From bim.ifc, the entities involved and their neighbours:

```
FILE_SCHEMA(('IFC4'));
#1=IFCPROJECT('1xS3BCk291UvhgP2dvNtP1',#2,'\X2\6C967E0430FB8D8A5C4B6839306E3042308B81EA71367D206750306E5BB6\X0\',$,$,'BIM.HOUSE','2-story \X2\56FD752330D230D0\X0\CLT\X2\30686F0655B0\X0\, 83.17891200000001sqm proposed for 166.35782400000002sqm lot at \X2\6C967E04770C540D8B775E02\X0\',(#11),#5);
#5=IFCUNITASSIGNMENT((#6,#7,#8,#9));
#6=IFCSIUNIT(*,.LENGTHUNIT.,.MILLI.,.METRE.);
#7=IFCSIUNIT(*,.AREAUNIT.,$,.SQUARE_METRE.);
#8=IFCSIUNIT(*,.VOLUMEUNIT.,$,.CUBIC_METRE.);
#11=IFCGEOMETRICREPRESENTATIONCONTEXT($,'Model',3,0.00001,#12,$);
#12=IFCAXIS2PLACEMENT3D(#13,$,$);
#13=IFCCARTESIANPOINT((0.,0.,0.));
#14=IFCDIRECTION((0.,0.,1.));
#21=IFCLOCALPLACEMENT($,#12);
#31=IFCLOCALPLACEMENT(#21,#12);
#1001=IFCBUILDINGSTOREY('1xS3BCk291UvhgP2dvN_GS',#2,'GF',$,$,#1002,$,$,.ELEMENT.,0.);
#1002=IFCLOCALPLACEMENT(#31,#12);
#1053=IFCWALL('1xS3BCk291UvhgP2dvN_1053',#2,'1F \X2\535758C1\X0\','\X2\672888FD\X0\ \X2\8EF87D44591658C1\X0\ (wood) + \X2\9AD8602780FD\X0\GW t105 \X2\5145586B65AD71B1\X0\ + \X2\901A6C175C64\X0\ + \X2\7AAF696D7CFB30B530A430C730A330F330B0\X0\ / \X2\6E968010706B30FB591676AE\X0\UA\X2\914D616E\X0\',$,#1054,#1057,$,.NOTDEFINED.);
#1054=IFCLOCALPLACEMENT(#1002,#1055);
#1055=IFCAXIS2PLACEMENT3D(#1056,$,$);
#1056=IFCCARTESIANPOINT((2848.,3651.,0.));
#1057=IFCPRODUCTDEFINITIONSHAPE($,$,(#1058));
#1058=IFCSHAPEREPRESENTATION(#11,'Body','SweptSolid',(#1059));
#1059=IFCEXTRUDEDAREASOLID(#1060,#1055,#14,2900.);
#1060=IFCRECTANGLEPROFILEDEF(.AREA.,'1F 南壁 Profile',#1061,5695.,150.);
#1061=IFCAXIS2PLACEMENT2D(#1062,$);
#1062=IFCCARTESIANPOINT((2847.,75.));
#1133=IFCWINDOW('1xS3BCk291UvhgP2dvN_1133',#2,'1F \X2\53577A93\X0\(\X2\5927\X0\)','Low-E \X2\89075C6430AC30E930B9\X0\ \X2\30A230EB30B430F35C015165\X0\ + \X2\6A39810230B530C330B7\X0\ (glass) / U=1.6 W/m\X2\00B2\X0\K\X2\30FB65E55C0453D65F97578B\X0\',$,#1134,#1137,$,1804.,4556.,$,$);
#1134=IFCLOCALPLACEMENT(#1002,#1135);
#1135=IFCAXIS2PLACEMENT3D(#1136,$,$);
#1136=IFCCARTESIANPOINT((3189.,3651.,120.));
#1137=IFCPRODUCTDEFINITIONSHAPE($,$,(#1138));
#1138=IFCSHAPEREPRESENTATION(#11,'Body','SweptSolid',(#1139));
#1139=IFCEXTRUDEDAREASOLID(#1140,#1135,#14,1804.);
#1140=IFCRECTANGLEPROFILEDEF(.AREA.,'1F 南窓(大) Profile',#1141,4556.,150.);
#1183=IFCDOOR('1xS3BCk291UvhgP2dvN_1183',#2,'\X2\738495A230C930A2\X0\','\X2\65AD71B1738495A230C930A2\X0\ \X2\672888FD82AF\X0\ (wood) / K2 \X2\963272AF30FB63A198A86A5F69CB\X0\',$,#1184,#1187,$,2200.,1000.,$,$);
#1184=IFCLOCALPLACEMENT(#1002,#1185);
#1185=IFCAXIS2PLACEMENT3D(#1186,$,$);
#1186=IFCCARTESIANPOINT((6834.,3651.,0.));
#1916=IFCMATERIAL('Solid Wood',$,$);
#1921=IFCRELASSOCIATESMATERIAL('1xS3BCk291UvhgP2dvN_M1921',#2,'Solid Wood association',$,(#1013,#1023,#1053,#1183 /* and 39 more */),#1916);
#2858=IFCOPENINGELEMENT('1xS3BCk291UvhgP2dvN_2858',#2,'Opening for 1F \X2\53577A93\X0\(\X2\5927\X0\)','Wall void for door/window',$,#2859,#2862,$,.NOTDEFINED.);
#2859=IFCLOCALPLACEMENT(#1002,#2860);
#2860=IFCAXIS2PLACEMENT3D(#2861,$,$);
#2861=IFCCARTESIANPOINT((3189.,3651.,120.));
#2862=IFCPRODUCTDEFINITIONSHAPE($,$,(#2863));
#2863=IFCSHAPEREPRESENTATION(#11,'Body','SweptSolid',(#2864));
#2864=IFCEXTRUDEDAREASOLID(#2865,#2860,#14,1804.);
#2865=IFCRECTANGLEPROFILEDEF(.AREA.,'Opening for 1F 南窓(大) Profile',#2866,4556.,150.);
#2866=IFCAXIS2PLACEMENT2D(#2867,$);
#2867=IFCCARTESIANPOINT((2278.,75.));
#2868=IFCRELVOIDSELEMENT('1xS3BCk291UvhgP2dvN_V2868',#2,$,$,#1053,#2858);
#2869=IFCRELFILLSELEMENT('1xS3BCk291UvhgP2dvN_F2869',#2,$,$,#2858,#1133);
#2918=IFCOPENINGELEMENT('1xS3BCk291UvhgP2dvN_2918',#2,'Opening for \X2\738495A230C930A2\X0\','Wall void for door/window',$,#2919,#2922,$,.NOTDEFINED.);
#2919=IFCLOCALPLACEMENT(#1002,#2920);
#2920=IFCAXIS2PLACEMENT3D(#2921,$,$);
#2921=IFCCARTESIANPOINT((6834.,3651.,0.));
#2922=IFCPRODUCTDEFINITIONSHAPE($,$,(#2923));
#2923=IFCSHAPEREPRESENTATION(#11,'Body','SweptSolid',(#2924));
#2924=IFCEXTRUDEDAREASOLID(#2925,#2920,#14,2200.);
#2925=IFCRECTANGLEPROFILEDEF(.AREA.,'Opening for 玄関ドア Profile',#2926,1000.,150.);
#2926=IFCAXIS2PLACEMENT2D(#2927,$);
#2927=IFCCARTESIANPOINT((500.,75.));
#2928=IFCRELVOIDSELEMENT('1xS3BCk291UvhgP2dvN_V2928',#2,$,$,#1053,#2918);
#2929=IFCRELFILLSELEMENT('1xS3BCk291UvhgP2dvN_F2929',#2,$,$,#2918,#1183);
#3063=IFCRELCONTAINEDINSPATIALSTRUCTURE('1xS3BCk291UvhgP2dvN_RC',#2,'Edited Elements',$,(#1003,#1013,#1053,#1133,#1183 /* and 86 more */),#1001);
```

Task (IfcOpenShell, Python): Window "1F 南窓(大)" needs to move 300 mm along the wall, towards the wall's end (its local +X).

```python
import ifcopenshell
import ifcopenshell.api.geometry
import ifcopenshell.util.placement
import ifcopenshell.util.unit

model = ifcopenshell.open("bim.ifc")
unit_scale = ifcopenshell.util.unit.calculate_unit_scale(model)

window = model.by_id(1133)
opening = window.FillsVoids[0].RelatingOpeningElement
wall = opening.VoidsElements[0].RelatingBuildingElement

wall_matrix = ifcopenshell.util.placement.get_local_placement(wall.ObjectPlacement)
shift = wall_matrix[:3, 0] * 0.3 / unit_scale
before = ifcopenshell.util.placement.get_local_placement(window.ObjectPlacement)[:3, 3].copy()

# The window is not placed relative to its opening, so move both.
for product in (opening, window):
    matrix = ifcopenshell.util.placement.get_local_placement(product.ObjectPlacement)
    matrix[:3, 3] += shift
    ifcopenshell.api.geometry.edit_object_placement(model, product=product, matrix=matrix, is_si=False)

after = ifcopenshell.util.placement.get_local_placement(window.ObjectPlacement)[:3, 3]
print("window moved by", (after - before).round(3) + 0.0)

model.write("bim_updated.ifc")
```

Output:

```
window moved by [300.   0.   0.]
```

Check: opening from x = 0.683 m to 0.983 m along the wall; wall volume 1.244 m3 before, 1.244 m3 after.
